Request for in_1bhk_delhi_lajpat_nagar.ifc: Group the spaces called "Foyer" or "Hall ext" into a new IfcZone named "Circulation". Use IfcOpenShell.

First a look at what the model holds.

```python
import ifcopenshell

model = ifcopenshell.open("in_1bhk_delhi_lajpat_nagar.ifc")
print(model.schema)
seen = {}
for space in model.by_type("IfcSpace"):
    seen[space.LongName] = seen.get(space.LongName, 0) + 1
for name, count in sorted(seen.items(), key=str):
    print(count, "x", name)
print("zones:", [z.Name for z in model.by_type("IfcZone")][:20])
```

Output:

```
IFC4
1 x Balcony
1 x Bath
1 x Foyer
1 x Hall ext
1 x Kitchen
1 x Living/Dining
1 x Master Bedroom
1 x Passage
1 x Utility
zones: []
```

```python
import ifcopenshell
import ifcopenshell.api.group
import ifcopenshell.api.root

model = ifcopenshell.open("in_1bhk_delhi_lajpat_nagar.ifc")

names = {"Foyer", "Hall ext"}
spaces = [s for s in model.by_type("IfcSpace") if s.LongName in names]

zone = ifcopenshell.api.root.create_entity(model, ifc_class="IfcZone", name="Circulation")
ifcopenshell.api.group.assign_group(model, products=spaces, group=zone)
print(len(spaces), "spaces in", zone.Name)

model.write("in_1bhk_delhi_lajpat_nagar-out.ifc")
```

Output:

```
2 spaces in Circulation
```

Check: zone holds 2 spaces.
